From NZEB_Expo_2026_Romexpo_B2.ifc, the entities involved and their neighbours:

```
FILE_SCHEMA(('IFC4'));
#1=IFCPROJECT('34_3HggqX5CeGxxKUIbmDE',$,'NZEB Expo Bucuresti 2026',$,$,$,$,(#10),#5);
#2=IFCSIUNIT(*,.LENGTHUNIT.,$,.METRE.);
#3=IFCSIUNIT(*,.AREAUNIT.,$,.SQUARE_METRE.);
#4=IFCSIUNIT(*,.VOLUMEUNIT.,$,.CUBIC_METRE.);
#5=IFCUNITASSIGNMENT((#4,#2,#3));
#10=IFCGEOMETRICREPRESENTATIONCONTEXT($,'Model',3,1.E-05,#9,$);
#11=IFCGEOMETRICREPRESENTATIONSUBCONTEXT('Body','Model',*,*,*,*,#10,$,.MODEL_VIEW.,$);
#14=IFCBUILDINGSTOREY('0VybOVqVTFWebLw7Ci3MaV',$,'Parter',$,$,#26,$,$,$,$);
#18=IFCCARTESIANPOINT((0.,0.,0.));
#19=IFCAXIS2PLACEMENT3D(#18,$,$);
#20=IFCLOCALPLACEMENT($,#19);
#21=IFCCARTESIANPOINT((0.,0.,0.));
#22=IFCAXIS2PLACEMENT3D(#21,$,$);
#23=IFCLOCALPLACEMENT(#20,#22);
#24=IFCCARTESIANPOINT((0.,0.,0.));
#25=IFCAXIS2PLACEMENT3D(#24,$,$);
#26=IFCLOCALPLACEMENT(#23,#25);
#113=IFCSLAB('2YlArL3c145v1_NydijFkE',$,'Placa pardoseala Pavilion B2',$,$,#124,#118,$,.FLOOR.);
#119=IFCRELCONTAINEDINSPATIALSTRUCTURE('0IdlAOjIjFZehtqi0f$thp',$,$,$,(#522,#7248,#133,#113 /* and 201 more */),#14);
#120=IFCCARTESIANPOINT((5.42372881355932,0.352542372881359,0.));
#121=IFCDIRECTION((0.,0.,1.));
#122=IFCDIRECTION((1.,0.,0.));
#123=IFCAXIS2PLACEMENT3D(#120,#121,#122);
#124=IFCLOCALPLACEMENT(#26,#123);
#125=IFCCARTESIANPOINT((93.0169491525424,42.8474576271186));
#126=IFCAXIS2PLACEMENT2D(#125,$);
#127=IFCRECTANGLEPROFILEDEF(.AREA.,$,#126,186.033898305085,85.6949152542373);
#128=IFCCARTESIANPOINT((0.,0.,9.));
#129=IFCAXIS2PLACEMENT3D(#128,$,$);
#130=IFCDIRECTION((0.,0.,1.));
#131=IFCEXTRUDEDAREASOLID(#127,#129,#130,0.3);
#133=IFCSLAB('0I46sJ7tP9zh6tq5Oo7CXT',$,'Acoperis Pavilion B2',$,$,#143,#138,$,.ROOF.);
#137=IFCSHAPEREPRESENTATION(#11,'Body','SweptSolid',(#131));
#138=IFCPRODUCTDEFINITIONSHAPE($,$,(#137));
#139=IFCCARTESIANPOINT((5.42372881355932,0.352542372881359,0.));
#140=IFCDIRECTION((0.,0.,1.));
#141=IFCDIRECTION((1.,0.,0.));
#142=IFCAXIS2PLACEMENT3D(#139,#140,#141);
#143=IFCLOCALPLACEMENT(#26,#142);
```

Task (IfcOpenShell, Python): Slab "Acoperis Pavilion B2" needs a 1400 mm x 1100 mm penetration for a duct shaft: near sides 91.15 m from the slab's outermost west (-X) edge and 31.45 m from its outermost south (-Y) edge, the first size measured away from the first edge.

```python
import numpy as np
import ifcopenshell
import ifcopenshell.api.feature
import ifcopenshell.api.geometry
import ifcopenshell.api.root
import ifcopenshell.geom
import ifcopenshell.util.placement
import ifcopenshell.util.representation
import ifcopenshell.util.shape
import ifcopenshell.util.unit

model = ifcopenshell.open("NZEB_Expo_2026_Romexpo_B2.ifc")
unit_scale = ifcopenshell.util.unit.calculate_unit_scale(model)
settings = ifcopenshell.geom.settings()


def volume(element):
    """Net volume in cubic metres, openings subtracted."""
    shape = ifcopenshell.geom.create_shape(settings, element)
    return ifcopenshell.util.shape.get_volume(shape.geometry)


slab = model.by_id(133)
before = volume(slab)

# Extent in the slab's own axes, in metres. The edges named are its -X and -Y sides.
slab_shape = ifcopenshell.geom.create_shape(settings, slab)
vertices = ifcopenshell.util.shape.get_vertices(slab_shape.geometry)
x_min, y_min, bottom = vertices.min(axis=0)
top = vertices[:, 2].max()

opening = ifcopenshell.api.root.create_entity(model, ifc_class="IfcOpeningElement", name="Duct shaft opening", predefined_type="OPENING")
context = ifcopenshell.util.representation.get_context(model, "Model", "Body", "MODEL_VIEW")
width, depth = 1.4, 1.1
outline = [(0.0, 0.0), (width, 0.0), (width, depth), (0.0, depth), (0.0, 0.0)]
# Overshoot both faces by 50 mm so the cut is clean.
shape = ifcopenshell.api.geometry.add_slab_representation(
    model, context=context, depth=top - bottom + 0.1, polyline=outline
)
ifcopenshell.api.geometry.assign_representation(model, product=opening, representation=shape)

matrix = ifcopenshell.util.placement.get_local_placement(slab.ObjectPlacement)
matrix[:, 3] = matrix @ np.append(np.array([x_min + 91.15, y_min + 31.45, bottom - 0.05]) / unit_scale, 1.0)
ifcopenshell.api.geometry.edit_object_placement(model, product=opening, matrix=matrix, is_si=False)
ifcopenshell.api.feature.add_feature(model, feature=opening, element=slab)

after = volume(slab)

print(f"slab volume {before:.3f} -> {after:.3f} m3")

model.write("NZEB_Expo_2026_Romexpo_B2_v2.ifc")
```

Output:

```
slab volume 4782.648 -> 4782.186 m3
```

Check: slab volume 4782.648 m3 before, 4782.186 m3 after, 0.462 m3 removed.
